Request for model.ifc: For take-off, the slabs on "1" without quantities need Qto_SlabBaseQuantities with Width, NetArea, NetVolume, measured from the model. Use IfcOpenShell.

First a look at what the model holds.

```python
import ifcopenshell
import ifcopenshell.util.element
import ifcopenshell.util.unit

model = ifcopenshell.open("model.ifc")
print(model.schema)
for unit_type in ("LENGTHUNIT", "AREAUNIT", "VOLUMEUNIT"):
    print(unit_type, ifcopenshell.util.unit.calculate_unit_scale(model, unit_type))
storey = next(s for s in model.by_type("IfcBuildingStorey") if s.Name == "1")
slabs = [e for e in ifcopenshell.util.element.get_decomposition(storey) if e.is_a("IfcSlab")]
for e in sorted(slabs, key=lambda e: e.id()):
    print(e.id(), e.is_a(), e.Name, list(ifcopenshell.util.element.get_psets(e, qtos_only=True)), sep=" | ")
```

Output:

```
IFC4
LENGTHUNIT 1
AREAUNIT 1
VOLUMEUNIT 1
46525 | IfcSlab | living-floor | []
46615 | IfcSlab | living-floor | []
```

```python
import ifcopenshell
import ifcopenshell.api.pset
import ifcopenshell.geom
import ifcopenshell.util.element
import ifcopenshell.util.shape
import ifcopenshell.util.unit

model = ifcopenshell.open("model.ifc")
unit_scale = ifcopenshell.util.unit.calculate_unit_scale(model)
area_scale = ifcopenshell.util.unit.calculate_unit_scale(model, "AREAUNIT")
volume_scale = ifcopenshell.util.unit.calculate_unit_scale(model, "VOLUMEUNIT")
settings = ifcopenshell.geom.settings()

storey = next(s for s in model.by_type("IfcBuildingStorey") if s.Name == "1")
slabs = [e for e in ifcopenshell.util.element.get_decomposition(storey) if e.is_a("IfcSlab")]

for e in sorted(slabs, key=lambda e: e.id()):
    if ifcopenshell.util.element.get_psets(e, qtos_only=True, should_inherit=False):
        continue
    # Geometry comes back in metres, in the element's own axes.
    shape = ifcopenshell.geom.create_shape(settings, e)
    values = {
        "Width": ifcopenshell.util.shape.get_z(shape.geometry) / unit_scale,
        "NetArea": ifcopenshell.util.shape.get_footprint_area(shape.geometry) / area_scale,
        "NetVolume": ifcopenshell.util.shape.get_volume(shape.geometry) / volume_scale,
    }
    qto = ifcopenshell.api.pset.add_qto(model, product=e, name="Qto_SlabBaseQuantities")
    ifcopenshell.api.pset.edit_qto(model, qto=qto, properties=values)
    print(e.id(), {k: round(v, 3) for k, v in values.items()})

model.write("model-out.ifc")
```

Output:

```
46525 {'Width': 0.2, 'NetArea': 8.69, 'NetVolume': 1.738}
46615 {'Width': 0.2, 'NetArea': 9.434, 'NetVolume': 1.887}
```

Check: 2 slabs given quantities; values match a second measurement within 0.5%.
